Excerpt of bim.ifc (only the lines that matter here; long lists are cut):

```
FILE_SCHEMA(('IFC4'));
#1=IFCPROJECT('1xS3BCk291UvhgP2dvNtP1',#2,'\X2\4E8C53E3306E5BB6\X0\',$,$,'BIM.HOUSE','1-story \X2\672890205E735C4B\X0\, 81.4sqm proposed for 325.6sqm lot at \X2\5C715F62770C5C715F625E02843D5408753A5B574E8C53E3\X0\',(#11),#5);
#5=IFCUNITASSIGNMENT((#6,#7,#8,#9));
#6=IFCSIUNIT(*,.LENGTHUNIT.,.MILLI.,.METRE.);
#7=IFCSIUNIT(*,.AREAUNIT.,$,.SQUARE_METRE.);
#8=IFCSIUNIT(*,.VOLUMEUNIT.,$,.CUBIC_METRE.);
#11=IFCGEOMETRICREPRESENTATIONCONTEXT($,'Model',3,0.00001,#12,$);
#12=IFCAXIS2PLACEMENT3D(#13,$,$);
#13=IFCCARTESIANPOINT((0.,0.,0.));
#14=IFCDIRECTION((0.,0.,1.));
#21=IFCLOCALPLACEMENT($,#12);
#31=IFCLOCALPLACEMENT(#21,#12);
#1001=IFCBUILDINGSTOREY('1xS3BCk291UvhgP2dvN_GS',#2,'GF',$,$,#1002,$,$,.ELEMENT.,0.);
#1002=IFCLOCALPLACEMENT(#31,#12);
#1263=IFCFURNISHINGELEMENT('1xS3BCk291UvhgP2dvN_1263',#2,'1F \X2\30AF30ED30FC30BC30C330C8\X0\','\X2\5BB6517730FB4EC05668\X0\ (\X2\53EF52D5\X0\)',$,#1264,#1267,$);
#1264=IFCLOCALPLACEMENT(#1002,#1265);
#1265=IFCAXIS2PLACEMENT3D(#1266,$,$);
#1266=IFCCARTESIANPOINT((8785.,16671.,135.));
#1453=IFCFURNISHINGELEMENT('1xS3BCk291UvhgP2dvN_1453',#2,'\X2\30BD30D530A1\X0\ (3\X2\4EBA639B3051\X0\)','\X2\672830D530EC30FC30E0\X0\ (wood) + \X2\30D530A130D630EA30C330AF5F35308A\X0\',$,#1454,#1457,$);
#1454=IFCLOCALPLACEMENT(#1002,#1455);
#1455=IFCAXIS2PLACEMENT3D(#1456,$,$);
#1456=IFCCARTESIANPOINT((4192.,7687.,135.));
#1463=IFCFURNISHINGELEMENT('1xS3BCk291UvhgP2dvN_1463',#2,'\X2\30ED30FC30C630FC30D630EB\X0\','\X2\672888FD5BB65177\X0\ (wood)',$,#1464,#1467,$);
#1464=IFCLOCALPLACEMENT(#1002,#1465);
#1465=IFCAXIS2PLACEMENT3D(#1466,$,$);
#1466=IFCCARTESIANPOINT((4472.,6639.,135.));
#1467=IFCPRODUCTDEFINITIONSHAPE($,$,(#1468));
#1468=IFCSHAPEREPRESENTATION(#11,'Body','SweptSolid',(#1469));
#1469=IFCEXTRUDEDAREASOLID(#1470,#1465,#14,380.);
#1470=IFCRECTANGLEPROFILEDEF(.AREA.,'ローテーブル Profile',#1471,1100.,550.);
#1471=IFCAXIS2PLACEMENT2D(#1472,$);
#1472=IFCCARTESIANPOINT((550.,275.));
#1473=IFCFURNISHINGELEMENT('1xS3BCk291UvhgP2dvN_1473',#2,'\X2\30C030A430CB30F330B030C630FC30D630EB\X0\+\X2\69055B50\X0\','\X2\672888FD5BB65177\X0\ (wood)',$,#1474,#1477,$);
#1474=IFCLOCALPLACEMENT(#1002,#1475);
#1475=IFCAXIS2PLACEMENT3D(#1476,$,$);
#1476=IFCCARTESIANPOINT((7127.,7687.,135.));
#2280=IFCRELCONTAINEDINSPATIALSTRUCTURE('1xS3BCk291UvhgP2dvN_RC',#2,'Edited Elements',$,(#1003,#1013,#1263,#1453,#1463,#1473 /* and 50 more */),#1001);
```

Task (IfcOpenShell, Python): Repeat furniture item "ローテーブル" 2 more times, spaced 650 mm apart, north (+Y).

```python
import numpy as np
import ifcopenshell
import ifcopenshell.api.geometry
import ifcopenshell.api.root
import ifcopenshell.util.element
import ifcopenshell.util.placement

model = ifcopenshell.open("bim.ifc")


def reuse_history(source, copy):
    """copy_class also copies each property set's owner history, people and application; keep the originals."""
    for rel in copy.IsDefinedBy:
        if rel.is_a("IfcRelDefinesByProperties") and (history := rel.RelatingPropertyDefinition.OwnerHistory):
            rel.RelatingPropertyDefinition.OwnerHistory = source.OwnerHistory
            ifcopenshell.util.element.remove_deep2(model, history)


source = model.by_id(1463)
base = ifcopenshell.util.placement.get_local_placement(source.ObjectPlacement)
step = np.array([0.0, 1.0, 0.0]) * 650.0

for i in range(1, 3):
    copy = ifcopenshell.api.root.copy_class(model, product=source)
    copy.Representation = ifcopenshell.util.element.copy_deep(
        model, source.Representation, exclude=["IfcGeometricRepresentationContext", "IfcRepresentationMap"]
    )
    reuse_history(source, copy)
    matrix = base.copy()
    matrix[:3, 3] += i * step
    print("added at", matrix[:3, 3].round(3) + 0.0)
    ifcopenshell.api.geometry.edit_object_placement(model, product=copy, matrix=matrix, is_si=False)

model.write("bim_updated.ifc")
```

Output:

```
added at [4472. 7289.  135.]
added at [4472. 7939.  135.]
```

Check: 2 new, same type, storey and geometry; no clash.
